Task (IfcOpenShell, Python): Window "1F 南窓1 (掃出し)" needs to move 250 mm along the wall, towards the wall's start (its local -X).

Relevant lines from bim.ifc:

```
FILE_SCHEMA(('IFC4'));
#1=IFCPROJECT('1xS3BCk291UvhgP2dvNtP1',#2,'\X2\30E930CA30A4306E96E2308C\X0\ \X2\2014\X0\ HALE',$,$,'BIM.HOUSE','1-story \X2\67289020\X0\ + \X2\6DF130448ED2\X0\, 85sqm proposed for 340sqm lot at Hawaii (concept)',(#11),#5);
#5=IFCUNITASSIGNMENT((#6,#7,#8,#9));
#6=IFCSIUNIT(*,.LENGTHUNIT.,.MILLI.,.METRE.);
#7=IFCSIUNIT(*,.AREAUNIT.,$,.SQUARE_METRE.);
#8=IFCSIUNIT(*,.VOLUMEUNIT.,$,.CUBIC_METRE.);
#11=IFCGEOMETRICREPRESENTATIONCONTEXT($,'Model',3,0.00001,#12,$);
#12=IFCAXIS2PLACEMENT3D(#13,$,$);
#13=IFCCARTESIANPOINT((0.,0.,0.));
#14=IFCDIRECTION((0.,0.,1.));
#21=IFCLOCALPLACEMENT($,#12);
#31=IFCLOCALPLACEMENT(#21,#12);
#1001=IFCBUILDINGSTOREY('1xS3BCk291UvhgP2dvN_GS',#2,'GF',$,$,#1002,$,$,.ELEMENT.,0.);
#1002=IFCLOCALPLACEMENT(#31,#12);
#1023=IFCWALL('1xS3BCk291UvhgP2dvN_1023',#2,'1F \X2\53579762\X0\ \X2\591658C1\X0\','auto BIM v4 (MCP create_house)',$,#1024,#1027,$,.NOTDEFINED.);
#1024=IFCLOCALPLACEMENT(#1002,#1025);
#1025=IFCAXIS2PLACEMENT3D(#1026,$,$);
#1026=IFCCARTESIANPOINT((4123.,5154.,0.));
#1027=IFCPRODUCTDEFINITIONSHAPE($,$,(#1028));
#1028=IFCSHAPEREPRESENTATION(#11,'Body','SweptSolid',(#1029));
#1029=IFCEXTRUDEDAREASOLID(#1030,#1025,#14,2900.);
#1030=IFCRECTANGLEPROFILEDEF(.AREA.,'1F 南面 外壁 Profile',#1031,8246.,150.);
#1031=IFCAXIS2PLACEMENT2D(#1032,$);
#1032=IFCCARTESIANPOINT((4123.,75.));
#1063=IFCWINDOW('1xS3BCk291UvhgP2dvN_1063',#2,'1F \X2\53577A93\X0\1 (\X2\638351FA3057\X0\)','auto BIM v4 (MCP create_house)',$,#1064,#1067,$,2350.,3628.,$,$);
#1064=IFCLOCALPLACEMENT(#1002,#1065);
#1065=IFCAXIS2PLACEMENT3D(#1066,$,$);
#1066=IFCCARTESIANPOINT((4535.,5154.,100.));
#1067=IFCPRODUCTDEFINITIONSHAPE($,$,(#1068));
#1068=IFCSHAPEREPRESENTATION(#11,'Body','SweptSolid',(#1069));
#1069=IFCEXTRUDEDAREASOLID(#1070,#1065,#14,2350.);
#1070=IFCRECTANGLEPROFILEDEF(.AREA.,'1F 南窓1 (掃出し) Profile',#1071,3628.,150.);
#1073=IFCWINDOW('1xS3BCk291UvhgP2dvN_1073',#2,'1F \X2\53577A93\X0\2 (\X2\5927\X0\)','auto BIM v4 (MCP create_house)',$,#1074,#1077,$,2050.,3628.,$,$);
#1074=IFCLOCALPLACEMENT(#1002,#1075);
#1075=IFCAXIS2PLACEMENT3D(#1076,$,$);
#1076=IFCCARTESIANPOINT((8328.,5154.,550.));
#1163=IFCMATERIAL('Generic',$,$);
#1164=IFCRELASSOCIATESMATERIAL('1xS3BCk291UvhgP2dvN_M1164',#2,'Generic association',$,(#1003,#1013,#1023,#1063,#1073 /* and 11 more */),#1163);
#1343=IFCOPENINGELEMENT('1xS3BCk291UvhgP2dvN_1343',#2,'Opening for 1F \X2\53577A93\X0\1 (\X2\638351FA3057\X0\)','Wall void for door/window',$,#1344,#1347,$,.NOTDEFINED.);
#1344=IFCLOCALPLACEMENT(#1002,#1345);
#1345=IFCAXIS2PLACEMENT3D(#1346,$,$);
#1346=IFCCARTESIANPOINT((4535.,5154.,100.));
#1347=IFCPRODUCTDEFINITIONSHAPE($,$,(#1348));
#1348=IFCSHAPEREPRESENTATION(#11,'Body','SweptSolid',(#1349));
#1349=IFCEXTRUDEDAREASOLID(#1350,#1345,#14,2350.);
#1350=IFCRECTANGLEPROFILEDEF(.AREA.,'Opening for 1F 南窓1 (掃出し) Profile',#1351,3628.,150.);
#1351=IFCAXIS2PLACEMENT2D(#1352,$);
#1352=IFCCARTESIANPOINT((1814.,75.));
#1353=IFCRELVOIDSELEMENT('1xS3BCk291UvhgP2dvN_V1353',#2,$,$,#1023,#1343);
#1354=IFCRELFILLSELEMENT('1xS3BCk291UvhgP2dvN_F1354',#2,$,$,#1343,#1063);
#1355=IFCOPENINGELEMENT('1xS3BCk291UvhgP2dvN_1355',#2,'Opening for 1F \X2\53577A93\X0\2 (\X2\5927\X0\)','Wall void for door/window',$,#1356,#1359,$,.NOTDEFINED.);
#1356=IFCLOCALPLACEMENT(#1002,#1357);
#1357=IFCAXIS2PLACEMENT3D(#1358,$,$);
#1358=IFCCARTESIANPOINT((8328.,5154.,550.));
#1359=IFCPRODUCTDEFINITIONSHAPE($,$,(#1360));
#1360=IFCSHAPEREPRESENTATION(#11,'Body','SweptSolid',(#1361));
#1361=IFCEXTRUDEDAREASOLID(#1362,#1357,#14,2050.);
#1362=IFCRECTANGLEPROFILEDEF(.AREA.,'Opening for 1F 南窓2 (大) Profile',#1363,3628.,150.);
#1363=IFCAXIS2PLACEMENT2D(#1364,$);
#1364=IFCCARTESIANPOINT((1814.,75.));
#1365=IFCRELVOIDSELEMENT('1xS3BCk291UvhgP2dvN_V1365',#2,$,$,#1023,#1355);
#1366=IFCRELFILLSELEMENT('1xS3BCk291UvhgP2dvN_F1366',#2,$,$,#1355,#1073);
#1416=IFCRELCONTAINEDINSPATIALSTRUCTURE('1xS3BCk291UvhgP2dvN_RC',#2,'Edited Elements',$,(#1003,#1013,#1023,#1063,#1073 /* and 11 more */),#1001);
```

```python
import ifcopenshell
import ifcopenshell.api.geometry
import ifcopenshell.util.placement
import ifcopenshell.util.unit

model = ifcopenshell.open("bim.ifc")
unit_scale = ifcopenshell.util.unit.calculate_unit_scale(model)

window = model.by_guid("1xS3BCk291UvhgP2dvN_1063")
opening = window.FillsVoids[0].RelatingOpeningElement
wall = opening.VoidsElements[0].RelatingBuildingElement

wall_matrix = ifcopenshell.util.placement.get_local_placement(wall.ObjectPlacement)
shift = wall_matrix[:3, 0] * -0.25 / unit_scale
before = ifcopenshell.util.placement.get_local_placement(window.ObjectPlacement)[:3, 3].copy()

# The window is not placed relative to its opening, so move both.
for product in (opening, window):
    matrix = ifcopenshell.util.placement.get_local_placement(product.ObjectPlacement)
    matrix[:3, 3] += shift
    ifcopenshell.api.geometry.edit_object_placement(model, product=product, matrix=matrix, is_si=False)

after = ifcopenshell.util.placement.get_local_placement(window.ObjectPlacement)[:3, 3]
print("window moved by", (after - before).round(3) + 0.0)

model.write("bim_updated.ifc")
```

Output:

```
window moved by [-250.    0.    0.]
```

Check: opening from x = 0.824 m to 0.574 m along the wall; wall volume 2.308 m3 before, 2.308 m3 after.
